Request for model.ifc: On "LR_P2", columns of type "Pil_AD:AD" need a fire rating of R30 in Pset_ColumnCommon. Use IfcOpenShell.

First a look at what the model holds.

```python
import ifcopenshell
import ifcopenshell.util.element

model = ifcopenshell.open("model.ifc")
print(model.schema)
storey = next(s for s in model.by_type("IfcBuildingStorey") if s.Name == "LR_P2")
columns = [e for e in ifcopenshell.util.element.get_decomposition(storey) if e.is_a("IfcColumn")]
seen = {}
for e in columns:
    element_type = ifcopenshell.util.element.get_type(e)
    key = (element_type.Name if element_type != e and element_type else None, ifcopenshell.util.element.get_pset(e, "Pset_ColumnCommon", "FireRating"))
    seen[key] = seen.get(key, 0) + 1
for (name, value), count in sorted(seen.items(), key=str):
    print(count, "x", name, "|", value)
```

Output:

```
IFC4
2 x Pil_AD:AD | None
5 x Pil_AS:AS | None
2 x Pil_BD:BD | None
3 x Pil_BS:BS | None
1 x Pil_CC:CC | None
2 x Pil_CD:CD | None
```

```python
import ifcopenshell
import ifcopenshell.api.pset
import ifcopenshell.util.element

model = ifcopenshell.open("model.ifc")

storey = next(s for s in model.by_type("IfcBuildingStorey") if s.Name == "LR_P2")
columns = [e for e in ifcopenshell.util.element.get_decomposition(storey) if e.is_a("IfcColumn")]

count = 0
for e in columns:
    element_type = ifcopenshell.util.element.get_type(e)
    if element_type in (None, e) or element_type.Name != "Pil_AD:AD":
        continue
    # add_pset returns the element's existing set when there is one.
    pset = ifcopenshell.api.pset.add_pset(model, product=e, name="Pset_ColumnCommon")
    ifcopenshell.api.pset.edit_pset(model, pset=pset, properties={"FireRating": "R30"})
    count += 1

print(count, "columns updated")

model.write("model_updated.ifc")
```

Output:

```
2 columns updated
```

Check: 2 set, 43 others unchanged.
